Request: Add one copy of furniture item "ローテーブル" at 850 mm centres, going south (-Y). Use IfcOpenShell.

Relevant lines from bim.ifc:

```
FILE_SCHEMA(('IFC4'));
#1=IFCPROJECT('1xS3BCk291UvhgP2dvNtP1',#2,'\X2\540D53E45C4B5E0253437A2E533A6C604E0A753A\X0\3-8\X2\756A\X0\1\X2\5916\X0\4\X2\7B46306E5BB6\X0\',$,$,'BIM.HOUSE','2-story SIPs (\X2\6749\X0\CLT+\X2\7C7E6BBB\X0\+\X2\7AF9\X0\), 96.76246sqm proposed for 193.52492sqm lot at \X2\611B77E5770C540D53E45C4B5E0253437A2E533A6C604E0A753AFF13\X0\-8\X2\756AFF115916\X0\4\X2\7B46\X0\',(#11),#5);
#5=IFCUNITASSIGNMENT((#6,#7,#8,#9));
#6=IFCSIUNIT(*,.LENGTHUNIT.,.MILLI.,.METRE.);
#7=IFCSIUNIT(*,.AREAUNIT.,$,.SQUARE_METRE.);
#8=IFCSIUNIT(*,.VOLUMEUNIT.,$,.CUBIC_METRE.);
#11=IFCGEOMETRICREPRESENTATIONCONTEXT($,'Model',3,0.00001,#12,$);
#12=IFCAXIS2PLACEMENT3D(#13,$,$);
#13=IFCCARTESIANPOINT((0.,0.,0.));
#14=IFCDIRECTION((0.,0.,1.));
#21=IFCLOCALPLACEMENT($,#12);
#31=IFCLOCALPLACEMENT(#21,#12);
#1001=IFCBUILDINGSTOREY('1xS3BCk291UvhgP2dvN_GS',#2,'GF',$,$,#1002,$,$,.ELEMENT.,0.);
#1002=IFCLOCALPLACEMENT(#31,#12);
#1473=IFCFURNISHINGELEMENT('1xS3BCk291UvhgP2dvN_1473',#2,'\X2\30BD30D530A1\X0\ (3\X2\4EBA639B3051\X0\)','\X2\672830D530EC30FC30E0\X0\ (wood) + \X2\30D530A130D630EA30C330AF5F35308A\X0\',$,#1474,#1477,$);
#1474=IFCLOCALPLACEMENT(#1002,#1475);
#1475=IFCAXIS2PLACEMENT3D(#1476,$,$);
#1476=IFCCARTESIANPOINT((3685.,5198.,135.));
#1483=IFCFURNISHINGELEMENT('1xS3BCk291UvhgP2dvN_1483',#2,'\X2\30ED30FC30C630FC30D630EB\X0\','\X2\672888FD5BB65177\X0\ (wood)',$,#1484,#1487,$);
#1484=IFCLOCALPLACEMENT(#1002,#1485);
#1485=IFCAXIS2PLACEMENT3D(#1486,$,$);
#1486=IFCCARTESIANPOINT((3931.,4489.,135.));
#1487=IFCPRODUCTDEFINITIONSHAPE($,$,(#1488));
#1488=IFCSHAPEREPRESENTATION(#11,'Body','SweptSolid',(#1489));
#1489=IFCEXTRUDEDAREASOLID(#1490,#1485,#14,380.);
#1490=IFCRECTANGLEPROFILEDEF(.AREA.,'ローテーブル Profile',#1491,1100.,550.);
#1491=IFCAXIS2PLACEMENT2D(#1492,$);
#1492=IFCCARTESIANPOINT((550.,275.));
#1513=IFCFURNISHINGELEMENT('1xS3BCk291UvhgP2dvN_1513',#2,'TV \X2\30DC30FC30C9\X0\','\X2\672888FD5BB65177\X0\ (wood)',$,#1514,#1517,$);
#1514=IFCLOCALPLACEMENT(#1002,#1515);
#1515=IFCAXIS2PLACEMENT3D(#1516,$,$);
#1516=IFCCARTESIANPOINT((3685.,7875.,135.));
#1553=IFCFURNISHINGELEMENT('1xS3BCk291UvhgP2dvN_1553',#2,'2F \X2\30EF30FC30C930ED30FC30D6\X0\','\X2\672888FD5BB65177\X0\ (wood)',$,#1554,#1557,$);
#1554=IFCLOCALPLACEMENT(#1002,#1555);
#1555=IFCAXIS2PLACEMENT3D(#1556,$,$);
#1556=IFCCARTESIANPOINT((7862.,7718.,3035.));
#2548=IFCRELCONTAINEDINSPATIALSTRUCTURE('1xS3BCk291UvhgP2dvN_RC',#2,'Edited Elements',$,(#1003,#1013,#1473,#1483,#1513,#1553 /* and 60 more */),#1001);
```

```python
import numpy as np
import ifcopenshell
import ifcopenshell.api.geometry
import ifcopenshell.api.root
import ifcopenshell.util.element
import ifcopenshell.util.placement

model = ifcopenshell.open("bim.ifc")


def reuse_history(source, copy):
    """copy_class also copies each property set's owner history, people and application; keep the originals."""
    for rel in copy.IsDefinedBy:
        if rel.is_a("IfcRelDefinesByProperties") and (history := rel.RelatingPropertyDefinition.OwnerHistory):
            rel.RelatingPropertyDefinition.OwnerHistory = source.OwnerHistory
            ifcopenshell.util.element.remove_deep2(model, history)


source = model.by_guid("1xS3BCk291UvhgP2dvN_1483")
base = ifcopenshell.util.placement.get_local_placement(source.ObjectPlacement)
step = np.array([0.0, -1.0, 0.0]) * 850.0

for i in range(1, 2):
    copy = ifcopenshell.api.root.copy_class(model, product=source)
    copy.Representation = ifcopenshell.util.element.copy_deep(
        model, source.Representation, exclude=["IfcGeometricRepresentationContext", "IfcRepresentationMap"]
    )
    reuse_history(source, copy)
    matrix = base.copy()
    matrix[:3, 3] += i * step
    print("added at", matrix[:3, 3].round(3) + 0.0)
    ifcopenshell.api.geometry.edit_object_placement(model, product=copy, matrix=matrix, is_si=False)

model.write("bim_v2.ifc")
```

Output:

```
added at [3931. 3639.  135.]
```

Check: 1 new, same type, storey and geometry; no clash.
